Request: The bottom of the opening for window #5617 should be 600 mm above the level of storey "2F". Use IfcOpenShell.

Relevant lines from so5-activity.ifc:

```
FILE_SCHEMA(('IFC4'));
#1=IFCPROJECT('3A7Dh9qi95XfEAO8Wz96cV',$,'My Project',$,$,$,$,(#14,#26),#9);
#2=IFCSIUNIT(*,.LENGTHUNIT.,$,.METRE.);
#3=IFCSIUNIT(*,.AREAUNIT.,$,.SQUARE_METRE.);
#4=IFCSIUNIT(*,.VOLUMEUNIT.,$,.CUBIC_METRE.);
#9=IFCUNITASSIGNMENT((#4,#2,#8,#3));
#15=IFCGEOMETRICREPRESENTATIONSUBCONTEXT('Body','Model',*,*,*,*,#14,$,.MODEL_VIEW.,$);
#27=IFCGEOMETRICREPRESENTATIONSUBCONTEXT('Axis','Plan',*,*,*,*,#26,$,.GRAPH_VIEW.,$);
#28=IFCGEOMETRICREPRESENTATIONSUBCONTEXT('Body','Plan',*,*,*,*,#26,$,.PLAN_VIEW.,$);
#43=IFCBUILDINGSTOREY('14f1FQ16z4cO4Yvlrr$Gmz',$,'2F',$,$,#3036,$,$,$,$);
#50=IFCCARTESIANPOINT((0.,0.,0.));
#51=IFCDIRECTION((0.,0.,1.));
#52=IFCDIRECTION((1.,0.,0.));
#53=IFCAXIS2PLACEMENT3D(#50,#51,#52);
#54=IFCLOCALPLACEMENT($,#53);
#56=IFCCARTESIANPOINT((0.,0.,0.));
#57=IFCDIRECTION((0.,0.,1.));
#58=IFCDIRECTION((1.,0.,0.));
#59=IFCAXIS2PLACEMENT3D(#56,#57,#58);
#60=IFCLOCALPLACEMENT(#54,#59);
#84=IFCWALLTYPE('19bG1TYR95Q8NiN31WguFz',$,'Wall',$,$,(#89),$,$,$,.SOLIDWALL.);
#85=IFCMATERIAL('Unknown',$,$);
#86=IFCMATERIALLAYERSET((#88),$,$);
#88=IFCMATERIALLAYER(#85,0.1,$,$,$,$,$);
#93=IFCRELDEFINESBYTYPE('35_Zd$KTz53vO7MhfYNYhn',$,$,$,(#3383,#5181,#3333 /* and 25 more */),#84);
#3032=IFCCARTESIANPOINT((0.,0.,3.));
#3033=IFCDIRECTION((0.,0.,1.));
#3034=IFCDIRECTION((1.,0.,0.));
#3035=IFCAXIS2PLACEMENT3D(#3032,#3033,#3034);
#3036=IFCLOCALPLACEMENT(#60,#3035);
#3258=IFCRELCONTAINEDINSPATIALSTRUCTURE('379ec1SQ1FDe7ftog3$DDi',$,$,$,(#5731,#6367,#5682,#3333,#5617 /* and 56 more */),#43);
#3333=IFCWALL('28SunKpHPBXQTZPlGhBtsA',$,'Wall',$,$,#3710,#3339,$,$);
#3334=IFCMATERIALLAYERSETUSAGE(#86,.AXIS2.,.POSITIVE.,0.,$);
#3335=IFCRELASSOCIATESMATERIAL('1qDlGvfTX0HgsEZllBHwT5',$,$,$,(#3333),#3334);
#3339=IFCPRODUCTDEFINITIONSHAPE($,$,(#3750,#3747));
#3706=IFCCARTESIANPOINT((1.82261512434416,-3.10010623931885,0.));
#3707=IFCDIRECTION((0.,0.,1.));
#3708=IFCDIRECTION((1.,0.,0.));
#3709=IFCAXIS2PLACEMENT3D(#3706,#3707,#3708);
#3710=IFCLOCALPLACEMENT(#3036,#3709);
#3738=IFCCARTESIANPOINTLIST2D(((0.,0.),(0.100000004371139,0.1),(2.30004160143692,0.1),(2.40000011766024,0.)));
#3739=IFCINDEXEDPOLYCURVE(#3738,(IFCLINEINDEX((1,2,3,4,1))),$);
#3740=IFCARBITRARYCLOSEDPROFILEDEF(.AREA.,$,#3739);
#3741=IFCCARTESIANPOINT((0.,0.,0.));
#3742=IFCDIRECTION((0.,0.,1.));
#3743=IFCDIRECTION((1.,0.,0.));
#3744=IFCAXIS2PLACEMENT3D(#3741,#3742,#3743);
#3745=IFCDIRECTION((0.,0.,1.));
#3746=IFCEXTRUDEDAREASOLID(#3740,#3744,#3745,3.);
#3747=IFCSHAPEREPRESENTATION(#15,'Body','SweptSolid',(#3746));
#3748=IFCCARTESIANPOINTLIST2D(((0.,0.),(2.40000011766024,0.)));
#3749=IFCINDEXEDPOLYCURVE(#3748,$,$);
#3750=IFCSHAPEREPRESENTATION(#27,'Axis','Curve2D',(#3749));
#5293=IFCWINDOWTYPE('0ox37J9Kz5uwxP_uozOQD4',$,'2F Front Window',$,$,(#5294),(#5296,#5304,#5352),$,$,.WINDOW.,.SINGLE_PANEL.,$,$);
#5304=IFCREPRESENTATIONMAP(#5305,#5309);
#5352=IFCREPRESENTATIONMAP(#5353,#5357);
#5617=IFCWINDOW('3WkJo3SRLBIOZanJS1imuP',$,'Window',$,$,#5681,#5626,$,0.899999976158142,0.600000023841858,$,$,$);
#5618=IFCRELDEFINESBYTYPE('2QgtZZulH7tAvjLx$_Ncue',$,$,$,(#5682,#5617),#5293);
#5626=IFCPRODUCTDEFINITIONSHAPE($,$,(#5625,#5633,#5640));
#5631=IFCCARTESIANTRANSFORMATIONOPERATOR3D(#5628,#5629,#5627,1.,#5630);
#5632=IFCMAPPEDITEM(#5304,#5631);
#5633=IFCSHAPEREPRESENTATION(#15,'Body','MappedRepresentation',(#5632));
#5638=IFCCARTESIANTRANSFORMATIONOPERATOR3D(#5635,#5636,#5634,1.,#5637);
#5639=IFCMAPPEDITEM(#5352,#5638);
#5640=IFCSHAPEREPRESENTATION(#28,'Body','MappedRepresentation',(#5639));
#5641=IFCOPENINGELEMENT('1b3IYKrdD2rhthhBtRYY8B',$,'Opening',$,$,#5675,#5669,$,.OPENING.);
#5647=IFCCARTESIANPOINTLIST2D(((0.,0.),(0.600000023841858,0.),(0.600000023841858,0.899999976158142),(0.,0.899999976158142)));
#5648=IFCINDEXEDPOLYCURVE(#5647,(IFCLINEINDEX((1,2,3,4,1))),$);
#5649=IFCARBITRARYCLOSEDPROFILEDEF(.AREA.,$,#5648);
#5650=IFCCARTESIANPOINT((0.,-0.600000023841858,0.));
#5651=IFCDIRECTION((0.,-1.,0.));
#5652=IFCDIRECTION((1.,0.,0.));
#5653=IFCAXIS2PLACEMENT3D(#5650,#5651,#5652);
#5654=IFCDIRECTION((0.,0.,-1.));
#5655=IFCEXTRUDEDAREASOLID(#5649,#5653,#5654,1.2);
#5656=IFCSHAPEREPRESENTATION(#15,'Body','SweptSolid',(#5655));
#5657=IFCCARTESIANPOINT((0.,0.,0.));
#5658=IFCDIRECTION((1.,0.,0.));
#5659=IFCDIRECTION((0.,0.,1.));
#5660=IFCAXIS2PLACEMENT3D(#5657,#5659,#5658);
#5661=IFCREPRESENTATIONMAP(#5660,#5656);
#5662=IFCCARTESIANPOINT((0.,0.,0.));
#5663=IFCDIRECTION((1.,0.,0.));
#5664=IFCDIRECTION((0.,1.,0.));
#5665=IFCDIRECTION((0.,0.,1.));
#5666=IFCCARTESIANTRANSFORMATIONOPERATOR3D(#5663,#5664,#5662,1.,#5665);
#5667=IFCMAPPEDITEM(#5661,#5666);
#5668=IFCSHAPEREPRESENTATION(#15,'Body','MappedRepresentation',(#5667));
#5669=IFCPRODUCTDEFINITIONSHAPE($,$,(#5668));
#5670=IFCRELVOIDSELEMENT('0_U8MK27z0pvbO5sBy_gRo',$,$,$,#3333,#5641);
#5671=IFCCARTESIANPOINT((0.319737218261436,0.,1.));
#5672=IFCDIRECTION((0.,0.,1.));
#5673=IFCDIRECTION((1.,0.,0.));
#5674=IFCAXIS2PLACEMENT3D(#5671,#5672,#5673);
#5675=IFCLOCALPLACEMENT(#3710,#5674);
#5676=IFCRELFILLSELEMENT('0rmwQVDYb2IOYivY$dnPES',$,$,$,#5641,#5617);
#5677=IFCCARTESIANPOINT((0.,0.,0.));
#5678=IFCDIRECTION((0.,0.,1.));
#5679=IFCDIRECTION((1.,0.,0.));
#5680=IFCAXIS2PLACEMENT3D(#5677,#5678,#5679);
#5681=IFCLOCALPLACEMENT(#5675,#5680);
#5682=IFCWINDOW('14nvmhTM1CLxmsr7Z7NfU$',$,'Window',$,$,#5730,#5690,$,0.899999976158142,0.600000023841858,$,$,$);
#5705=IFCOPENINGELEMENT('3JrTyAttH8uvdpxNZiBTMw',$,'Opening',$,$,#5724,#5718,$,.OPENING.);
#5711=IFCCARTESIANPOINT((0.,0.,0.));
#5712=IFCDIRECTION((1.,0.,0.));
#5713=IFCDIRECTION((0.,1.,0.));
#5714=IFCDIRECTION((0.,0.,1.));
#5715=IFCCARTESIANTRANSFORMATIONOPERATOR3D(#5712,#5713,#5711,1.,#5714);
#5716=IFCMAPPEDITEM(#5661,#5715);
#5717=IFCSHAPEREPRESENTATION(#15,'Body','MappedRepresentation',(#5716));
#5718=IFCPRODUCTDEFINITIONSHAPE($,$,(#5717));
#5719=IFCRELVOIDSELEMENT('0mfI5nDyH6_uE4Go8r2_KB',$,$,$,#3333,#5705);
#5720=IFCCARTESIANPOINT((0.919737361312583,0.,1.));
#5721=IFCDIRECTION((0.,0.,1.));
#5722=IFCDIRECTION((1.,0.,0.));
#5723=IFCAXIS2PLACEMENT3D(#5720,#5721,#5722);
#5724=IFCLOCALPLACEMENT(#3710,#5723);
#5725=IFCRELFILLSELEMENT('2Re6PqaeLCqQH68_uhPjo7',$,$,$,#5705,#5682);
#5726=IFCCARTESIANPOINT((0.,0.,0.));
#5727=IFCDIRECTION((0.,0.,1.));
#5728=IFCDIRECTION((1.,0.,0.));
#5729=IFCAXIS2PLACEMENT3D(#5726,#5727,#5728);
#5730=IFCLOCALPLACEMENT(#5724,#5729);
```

```python
import numpy as np
import ifcopenshell
import ifcopenshell.api.geometry
import ifcopenshell.geom
import ifcopenshell.util.element
import ifcopenshell.util.placement
import ifcopenshell.util.shape
import ifcopenshell.util.unit

model = ifcopenshell.open("so5-activity.ifc")
unit_scale = ifcopenshell.util.unit.calculate_unit_scale(model)

window = model.by_guid("3WkJo3SRLBIOZanJS1imuP")
opening = window.FillsVoids[0].RelatingOpeningElement
storey = ifcopenshell.util.element.get_container(window, ifc_class="IfcBuildingStorey")
level = ifcopenshell.util.placement.get_local_placement(storey.ObjectPlacement)[2, 3]

# The opening's origin need not be at the sill, so measure its lowest point.
shape = ifcopenshell.geom.create_shape(ifcopenshell.geom.settings(), opening)
bottom = ifcopenshell.util.shape.get_shape_bottom_elevation(shape, shape.geometry) / unit_scale
dz = level + 0.6 / unit_scale - bottom

shift = np.array([0.0, 0.0, dz])
# The window is placed relative to its opening, so it follows when the opening moves.
matrix = ifcopenshell.util.placement.get_local_placement(opening.ObjectPlacement)
matrix[:3, 3] += shift
ifcopenshell.api.geometry.edit_object_placement(
    model, product=opening, matrix=matrix, is_si=False, should_transform_children=True
)

print(f"moved by {dz * unit_scale:+.3f} m")

model.write("so5-activity_rev.ifc")
```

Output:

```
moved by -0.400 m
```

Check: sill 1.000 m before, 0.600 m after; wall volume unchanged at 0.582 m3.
